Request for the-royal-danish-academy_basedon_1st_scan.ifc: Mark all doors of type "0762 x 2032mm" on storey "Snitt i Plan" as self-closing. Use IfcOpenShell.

First a look at what the model holds.

```python
import ifcopenshell
import ifcopenshell.util.element

model = ifcopenshell.open("the-royal-danish-academy_basedon_1st_scan.ifc")
print(model.schema)
storey = next(s for s in model.by_type("IfcBuildingStorey") if s.Name == "Snitt i Plan")
doors = [e for e in ifcopenshell.util.element.get_decomposition(storey) if e.is_a("IfcDoor")]
seen = {}
for e in doors:
    element_type = ifcopenshell.util.element.get_type(e)
    key = (element_type.Name if element_type != e and element_type else None, ifcopenshell.util.element.get_pset(e, "Pset_DoorCommon", "SelfClosing"))
    seen[key] = seen.get(key, 0) + 1
for (name, value), count in sorted(seen.items(), key=str):
    print(count, "x", name, "|", value)
```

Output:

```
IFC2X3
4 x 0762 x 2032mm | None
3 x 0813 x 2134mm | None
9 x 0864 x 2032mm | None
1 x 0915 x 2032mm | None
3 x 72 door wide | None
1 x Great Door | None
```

```python
import ifcopenshell
import ifcopenshell.api.pset
import ifcopenshell.util.element

model = ifcopenshell.open("the-royal-danish-academy_basedon_1st_scan.ifc")

storey = next(s for s in model.by_type("IfcBuildingStorey") if s.Name == "Snitt i Plan")
doors = [e for e in ifcopenshell.util.element.get_decomposition(storey) if e.is_a("IfcDoor")]

count = 0
for e in doors:
    element_type = ifcopenshell.util.element.get_type(e)
    if element_type in (None, e) or element_type.Name != "0762 x 2032mm":
        continue
    # add_pset returns the element's existing set when there is one.
    pset = ifcopenshell.api.pset.add_pset(model, product=e, name="Pset_DoorCommon")
    ifcopenshell.api.pset.edit_pset(model, pset=pset, properties={"SelfClosing": True})
    count += 1

print(count, "doors updated")

model.write("the-royal-danish-academy_basedon_1st_scan-out.ifc")
```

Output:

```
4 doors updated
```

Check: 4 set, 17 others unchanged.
